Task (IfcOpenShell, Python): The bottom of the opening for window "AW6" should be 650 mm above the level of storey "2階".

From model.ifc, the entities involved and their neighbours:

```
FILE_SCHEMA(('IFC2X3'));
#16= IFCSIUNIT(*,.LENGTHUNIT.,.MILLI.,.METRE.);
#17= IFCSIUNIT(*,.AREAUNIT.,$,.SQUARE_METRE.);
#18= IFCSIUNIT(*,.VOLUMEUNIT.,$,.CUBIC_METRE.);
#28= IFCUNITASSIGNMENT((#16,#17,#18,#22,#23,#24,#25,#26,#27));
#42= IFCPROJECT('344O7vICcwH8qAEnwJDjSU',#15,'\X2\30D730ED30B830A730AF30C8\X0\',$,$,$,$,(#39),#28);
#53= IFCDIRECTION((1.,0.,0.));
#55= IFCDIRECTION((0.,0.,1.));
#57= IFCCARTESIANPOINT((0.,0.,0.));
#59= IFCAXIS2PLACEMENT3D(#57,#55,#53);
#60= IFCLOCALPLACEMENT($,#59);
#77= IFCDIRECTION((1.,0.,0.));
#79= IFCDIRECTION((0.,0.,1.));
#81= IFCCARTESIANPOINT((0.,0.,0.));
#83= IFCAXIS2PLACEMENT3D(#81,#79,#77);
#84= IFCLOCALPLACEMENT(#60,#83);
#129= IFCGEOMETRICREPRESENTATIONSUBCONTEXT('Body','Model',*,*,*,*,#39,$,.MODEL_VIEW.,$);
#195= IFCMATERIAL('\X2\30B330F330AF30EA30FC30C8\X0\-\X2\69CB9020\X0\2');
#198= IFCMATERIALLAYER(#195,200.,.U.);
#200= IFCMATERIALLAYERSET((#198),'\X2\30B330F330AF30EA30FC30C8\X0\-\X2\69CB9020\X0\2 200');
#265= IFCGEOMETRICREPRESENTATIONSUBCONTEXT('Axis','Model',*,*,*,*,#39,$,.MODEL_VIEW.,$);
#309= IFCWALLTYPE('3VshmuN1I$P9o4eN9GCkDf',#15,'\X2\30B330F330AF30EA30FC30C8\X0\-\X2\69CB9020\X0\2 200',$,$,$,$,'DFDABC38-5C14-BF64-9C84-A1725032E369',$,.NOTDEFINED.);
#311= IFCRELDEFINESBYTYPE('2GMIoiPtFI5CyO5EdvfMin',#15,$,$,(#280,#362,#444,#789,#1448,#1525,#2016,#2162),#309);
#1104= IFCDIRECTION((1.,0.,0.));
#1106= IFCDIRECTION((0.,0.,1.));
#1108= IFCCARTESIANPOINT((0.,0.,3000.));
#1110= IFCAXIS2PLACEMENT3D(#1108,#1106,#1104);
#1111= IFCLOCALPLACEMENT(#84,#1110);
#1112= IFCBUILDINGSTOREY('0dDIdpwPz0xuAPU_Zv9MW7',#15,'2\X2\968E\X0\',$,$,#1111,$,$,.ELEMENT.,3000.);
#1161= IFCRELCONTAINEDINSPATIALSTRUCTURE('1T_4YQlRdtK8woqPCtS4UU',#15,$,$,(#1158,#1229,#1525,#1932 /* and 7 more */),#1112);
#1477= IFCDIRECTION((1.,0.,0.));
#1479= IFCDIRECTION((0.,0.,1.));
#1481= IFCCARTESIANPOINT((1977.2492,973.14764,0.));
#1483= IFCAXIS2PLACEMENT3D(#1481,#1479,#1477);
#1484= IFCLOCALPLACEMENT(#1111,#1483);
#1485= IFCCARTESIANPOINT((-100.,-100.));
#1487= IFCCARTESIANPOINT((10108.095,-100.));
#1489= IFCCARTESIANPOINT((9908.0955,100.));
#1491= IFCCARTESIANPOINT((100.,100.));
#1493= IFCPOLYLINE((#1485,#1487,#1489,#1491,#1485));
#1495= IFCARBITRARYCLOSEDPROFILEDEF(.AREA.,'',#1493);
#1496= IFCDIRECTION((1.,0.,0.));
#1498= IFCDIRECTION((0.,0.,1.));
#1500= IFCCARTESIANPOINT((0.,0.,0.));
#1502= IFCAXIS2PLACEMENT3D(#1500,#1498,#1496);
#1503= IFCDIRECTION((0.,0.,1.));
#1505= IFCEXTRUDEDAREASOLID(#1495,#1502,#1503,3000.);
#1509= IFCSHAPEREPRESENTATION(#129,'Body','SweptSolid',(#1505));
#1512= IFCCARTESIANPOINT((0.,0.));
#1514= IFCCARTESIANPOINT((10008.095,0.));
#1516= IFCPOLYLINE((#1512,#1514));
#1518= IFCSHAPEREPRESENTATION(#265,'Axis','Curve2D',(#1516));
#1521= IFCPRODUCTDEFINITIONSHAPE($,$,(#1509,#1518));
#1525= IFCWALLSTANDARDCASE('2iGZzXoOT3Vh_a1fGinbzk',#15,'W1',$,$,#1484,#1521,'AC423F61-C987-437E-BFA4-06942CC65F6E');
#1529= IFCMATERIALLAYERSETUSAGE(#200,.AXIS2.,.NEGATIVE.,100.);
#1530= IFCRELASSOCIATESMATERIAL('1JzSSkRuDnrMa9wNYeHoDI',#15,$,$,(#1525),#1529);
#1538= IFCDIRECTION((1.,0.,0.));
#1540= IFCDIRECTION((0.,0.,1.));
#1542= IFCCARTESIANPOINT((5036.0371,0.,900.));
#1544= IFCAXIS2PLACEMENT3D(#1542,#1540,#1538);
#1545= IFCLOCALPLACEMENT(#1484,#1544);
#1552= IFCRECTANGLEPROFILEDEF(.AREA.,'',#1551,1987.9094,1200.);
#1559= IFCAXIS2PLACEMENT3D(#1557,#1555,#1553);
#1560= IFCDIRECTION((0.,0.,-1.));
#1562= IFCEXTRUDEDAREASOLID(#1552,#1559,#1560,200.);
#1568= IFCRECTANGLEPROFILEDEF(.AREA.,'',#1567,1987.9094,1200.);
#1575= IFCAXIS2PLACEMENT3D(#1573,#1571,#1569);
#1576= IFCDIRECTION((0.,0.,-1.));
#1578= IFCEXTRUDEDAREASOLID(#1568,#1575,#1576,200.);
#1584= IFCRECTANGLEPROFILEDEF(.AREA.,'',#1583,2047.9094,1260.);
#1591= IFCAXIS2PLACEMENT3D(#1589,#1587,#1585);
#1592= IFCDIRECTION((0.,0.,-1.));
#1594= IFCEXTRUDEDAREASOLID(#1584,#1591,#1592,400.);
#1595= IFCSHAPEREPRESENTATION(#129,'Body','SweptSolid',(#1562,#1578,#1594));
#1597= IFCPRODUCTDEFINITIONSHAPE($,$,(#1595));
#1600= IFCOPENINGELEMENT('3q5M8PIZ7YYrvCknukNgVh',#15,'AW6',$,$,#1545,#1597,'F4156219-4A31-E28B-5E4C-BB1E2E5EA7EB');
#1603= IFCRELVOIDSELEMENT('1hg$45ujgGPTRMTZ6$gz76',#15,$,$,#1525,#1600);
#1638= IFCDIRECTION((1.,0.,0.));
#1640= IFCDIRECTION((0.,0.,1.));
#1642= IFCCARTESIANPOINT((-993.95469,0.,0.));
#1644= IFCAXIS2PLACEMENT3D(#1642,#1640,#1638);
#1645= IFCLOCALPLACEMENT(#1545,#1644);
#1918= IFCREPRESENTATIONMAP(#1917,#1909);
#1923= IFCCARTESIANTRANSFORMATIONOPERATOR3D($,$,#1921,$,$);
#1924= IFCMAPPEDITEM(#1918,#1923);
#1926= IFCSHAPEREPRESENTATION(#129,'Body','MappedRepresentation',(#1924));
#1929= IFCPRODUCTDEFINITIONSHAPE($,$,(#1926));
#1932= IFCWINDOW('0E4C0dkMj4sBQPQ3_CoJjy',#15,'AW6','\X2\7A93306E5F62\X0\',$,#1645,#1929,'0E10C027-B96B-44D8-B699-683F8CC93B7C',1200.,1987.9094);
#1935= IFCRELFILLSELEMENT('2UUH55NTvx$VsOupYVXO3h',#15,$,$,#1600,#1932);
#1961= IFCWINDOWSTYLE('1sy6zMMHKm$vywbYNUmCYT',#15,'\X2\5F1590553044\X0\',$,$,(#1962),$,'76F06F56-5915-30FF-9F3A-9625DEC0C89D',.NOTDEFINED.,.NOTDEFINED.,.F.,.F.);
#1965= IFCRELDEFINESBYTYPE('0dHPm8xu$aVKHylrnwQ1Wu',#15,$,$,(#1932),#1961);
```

```python
import numpy as np
import ifcopenshell
import ifcopenshell.api.geometry
import ifcopenshell.geom
import ifcopenshell.util.element
import ifcopenshell.util.placement
import ifcopenshell.util.shape
import ifcopenshell.util.unit

model = ifcopenshell.open("model.ifc")
unit_scale = ifcopenshell.util.unit.calculate_unit_scale(model)

window = model.by_guid("0E4C0dkMj4sBQPQ3_CoJjy")
opening = window.FillsVoids[0].RelatingOpeningElement
storey = ifcopenshell.util.element.get_container(window, ifc_class="IfcBuildingStorey")
level = ifcopenshell.util.placement.get_local_placement(storey.ObjectPlacement)[2, 3]

# The opening's origin need not be at the sill, so measure its lowest point.
shape = ifcopenshell.geom.create_shape(ifcopenshell.geom.settings(), opening)
bottom = ifcopenshell.util.shape.get_shape_bottom_elevation(shape, shape.geometry) / unit_scale
dz = level + 0.65 / unit_scale - bottom

shift = np.array([0.0, 0.0, dz])
# The window is placed relative to its opening, so it follows when the opening moves.
matrix = ifcopenshell.util.placement.get_local_placement(opening.ObjectPlacement)
matrix[:3, 3] += shift
ifcopenshell.api.geometry.edit_object_placement(
    model, product=opening, matrix=matrix, is_si=False, should_transform_children=True
)

print(f"moved by {dz * unit_scale:+.3f} m")

model.write("model_v2.ifc")
```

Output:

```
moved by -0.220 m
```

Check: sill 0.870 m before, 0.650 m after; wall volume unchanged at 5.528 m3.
